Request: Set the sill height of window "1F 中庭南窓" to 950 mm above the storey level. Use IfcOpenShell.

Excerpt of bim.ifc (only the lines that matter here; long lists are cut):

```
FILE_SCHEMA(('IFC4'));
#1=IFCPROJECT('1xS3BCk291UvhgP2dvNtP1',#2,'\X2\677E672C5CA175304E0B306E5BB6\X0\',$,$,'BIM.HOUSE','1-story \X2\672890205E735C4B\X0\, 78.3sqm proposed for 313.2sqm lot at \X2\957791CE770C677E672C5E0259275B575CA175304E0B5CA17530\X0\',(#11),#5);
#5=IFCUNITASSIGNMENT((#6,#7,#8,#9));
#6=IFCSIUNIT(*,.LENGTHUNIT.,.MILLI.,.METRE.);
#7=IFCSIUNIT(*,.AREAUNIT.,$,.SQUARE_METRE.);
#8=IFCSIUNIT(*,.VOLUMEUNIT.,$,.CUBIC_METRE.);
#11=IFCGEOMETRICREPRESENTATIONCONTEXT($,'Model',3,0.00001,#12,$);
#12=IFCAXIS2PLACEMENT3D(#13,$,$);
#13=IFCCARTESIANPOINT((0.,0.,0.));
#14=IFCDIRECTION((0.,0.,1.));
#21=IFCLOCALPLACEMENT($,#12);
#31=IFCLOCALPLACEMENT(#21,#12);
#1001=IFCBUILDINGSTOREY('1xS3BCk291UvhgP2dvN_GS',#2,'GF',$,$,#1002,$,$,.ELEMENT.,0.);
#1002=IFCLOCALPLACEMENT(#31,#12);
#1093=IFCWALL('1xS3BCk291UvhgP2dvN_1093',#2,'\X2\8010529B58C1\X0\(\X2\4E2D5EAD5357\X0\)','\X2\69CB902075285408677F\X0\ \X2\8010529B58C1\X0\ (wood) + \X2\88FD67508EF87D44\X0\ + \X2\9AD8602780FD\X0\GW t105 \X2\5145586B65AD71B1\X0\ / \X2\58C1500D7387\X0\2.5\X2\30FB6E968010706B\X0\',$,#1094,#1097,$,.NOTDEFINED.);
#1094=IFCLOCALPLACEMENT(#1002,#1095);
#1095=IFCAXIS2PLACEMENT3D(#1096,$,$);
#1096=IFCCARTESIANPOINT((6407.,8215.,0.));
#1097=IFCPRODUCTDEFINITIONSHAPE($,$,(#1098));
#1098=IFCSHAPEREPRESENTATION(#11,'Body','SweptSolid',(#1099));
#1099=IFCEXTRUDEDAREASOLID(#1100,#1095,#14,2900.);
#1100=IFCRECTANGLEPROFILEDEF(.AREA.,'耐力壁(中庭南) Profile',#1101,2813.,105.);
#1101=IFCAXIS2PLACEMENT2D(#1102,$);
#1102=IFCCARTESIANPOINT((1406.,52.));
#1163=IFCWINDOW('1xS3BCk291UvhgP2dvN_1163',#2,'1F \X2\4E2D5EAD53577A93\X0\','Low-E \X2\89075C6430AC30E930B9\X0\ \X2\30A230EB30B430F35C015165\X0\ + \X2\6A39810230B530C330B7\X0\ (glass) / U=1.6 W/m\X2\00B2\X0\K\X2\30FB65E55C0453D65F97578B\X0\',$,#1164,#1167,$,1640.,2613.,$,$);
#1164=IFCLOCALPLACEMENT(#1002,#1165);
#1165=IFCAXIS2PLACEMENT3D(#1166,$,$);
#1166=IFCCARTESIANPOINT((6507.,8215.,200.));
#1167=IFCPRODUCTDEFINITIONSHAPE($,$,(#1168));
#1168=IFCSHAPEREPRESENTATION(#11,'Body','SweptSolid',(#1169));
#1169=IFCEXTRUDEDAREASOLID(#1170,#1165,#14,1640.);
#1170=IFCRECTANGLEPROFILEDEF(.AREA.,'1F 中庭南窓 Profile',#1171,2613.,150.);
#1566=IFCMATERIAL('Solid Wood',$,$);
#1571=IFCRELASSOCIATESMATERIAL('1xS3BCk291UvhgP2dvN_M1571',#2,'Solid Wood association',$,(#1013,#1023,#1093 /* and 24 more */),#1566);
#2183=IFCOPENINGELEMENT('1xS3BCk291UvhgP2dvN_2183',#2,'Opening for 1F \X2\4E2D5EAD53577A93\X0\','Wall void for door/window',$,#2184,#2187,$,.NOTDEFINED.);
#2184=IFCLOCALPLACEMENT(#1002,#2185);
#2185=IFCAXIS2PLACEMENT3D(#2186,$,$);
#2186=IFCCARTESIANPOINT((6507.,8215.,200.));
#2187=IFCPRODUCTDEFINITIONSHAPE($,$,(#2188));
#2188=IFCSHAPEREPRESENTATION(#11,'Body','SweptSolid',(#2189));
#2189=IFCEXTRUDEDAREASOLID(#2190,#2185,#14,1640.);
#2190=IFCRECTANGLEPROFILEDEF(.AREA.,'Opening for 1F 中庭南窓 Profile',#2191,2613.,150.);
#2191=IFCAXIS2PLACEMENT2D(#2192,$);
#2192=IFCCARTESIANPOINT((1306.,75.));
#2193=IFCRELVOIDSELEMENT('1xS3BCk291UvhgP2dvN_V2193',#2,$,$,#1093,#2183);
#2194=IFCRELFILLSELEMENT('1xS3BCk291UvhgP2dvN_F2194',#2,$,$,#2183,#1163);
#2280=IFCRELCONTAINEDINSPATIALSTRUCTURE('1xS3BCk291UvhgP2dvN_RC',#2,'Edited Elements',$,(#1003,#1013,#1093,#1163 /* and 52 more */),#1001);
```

```python
import numpy as np
import ifcopenshell
import ifcopenshell.api.geometry
import ifcopenshell.geom
import ifcopenshell.util.element
import ifcopenshell.util.placement
import ifcopenshell.util.shape
import ifcopenshell.util.unit

model = ifcopenshell.open("bim.ifc")
unit_scale = ifcopenshell.util.unit.calculate_unit_scale(model)

window = model.by_id(1163)
opening = window.FillsVoids[0].RelatingOpeningElement
storey = ifcopenshell.util.element.get_container(window, ifc_class="IfcBuildingStorey")
level = ifcopenshell.util.placement.get_local_placement(storey.ObjectPlacement)[2, 3]

# The opening's origin need not be at the sill, so measure its lowest point.
shape = ifcopenshell.geom.create_shape(ifcopenshell.geom.settings(), opening)
bottom = ifcopenshell.util.shape.get_shape_bottom_elevation(shape, shape.geometry) / unit_scale
dz = level + 0.95 / unit_scale - bottom

shift = np.array([0.0, 0.0, dz])
# The window is not placed relative to its opening, so move both.
for product in (opening, window):
    matrix = ifcopenshell.util.placement.get_local_placement(product.ObjectPlacement)
    matrix[:3, 3] += shift
    ifcopenshell.api.geometry.edit_object_placement(model, product=product, matrix=matrix, is_si=False)

print(f"moved by {dz * unit_scale:+.3f} m")

model.write("bim_updated.ifc")
```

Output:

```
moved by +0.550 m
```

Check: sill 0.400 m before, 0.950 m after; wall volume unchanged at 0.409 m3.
